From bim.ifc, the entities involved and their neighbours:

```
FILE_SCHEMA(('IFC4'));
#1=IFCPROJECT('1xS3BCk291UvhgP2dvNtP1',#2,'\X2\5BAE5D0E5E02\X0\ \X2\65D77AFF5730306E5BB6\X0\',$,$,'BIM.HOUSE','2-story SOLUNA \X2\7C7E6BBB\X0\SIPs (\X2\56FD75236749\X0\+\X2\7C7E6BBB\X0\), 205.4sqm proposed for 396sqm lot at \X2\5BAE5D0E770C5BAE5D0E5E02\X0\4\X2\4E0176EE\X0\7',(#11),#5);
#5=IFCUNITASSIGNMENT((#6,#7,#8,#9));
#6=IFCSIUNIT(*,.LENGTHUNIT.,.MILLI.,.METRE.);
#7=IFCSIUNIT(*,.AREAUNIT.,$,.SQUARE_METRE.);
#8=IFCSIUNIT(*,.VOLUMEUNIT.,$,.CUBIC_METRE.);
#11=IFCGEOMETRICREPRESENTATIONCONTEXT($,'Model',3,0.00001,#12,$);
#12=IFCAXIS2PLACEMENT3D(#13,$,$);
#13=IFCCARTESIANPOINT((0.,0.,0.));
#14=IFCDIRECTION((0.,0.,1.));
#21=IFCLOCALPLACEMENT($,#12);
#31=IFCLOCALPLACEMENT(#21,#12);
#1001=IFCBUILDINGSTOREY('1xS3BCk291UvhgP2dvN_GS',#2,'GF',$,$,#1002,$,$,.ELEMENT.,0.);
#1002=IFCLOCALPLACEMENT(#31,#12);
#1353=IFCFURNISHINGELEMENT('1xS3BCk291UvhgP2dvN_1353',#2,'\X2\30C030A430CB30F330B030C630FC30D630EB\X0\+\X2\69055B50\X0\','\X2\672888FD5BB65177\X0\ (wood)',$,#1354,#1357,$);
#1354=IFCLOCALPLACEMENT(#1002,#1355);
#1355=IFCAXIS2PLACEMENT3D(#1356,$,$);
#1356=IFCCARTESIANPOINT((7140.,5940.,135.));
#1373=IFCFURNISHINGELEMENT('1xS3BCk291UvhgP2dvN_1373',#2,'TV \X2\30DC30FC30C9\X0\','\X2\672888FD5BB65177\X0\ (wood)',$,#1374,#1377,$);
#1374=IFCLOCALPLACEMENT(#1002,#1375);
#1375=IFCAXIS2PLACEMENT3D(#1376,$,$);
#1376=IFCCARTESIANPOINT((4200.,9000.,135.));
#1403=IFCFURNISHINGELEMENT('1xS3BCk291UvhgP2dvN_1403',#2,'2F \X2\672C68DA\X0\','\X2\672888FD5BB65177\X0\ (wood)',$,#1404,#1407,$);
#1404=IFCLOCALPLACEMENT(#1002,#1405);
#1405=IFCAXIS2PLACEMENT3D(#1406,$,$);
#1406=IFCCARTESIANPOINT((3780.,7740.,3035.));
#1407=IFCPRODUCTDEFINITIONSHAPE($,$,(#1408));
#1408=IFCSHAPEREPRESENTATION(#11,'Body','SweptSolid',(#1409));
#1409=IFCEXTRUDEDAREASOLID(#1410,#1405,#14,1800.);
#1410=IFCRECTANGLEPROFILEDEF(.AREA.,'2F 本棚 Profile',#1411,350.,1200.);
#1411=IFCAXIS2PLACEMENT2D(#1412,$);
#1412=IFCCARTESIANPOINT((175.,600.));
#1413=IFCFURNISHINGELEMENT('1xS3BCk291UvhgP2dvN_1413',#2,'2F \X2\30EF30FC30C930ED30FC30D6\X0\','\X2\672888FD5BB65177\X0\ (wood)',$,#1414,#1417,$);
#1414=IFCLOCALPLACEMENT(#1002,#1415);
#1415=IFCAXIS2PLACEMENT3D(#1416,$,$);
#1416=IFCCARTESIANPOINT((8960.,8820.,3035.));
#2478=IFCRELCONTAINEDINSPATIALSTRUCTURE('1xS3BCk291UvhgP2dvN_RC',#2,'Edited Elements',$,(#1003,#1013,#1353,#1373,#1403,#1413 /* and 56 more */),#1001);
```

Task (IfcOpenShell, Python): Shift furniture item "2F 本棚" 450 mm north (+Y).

```python
import ifcopenshell
import ifcopenshell.api.geometry
import ifcopenshell.util.placement
import ifcopenshell.util.unit

model = ifcopenshell.open("bim.ifc")
unit_scale = ifcopenshell.util.unit.calculate_unit_scale(model)

item = model.by_id(1403)
matrix = ifcopenshell.util.placement.get_local_placement(item.ObjectPlacement)
matrix[1, 3] += 0.45 / unit_scale
ifcopenshell.api.geometry.edit_object_placement(model, product=item, matrix=matrix, is_si=False)

print(ifcopenshell.util.placement.get_local_placement(item.ObjectPlacement).round(3) + 0.0)

model.write("bim_rev.ifc")
```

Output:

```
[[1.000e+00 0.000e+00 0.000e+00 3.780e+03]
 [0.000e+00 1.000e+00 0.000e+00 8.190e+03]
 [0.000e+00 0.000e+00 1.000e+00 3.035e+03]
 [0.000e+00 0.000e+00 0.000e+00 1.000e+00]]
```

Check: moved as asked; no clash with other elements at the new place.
